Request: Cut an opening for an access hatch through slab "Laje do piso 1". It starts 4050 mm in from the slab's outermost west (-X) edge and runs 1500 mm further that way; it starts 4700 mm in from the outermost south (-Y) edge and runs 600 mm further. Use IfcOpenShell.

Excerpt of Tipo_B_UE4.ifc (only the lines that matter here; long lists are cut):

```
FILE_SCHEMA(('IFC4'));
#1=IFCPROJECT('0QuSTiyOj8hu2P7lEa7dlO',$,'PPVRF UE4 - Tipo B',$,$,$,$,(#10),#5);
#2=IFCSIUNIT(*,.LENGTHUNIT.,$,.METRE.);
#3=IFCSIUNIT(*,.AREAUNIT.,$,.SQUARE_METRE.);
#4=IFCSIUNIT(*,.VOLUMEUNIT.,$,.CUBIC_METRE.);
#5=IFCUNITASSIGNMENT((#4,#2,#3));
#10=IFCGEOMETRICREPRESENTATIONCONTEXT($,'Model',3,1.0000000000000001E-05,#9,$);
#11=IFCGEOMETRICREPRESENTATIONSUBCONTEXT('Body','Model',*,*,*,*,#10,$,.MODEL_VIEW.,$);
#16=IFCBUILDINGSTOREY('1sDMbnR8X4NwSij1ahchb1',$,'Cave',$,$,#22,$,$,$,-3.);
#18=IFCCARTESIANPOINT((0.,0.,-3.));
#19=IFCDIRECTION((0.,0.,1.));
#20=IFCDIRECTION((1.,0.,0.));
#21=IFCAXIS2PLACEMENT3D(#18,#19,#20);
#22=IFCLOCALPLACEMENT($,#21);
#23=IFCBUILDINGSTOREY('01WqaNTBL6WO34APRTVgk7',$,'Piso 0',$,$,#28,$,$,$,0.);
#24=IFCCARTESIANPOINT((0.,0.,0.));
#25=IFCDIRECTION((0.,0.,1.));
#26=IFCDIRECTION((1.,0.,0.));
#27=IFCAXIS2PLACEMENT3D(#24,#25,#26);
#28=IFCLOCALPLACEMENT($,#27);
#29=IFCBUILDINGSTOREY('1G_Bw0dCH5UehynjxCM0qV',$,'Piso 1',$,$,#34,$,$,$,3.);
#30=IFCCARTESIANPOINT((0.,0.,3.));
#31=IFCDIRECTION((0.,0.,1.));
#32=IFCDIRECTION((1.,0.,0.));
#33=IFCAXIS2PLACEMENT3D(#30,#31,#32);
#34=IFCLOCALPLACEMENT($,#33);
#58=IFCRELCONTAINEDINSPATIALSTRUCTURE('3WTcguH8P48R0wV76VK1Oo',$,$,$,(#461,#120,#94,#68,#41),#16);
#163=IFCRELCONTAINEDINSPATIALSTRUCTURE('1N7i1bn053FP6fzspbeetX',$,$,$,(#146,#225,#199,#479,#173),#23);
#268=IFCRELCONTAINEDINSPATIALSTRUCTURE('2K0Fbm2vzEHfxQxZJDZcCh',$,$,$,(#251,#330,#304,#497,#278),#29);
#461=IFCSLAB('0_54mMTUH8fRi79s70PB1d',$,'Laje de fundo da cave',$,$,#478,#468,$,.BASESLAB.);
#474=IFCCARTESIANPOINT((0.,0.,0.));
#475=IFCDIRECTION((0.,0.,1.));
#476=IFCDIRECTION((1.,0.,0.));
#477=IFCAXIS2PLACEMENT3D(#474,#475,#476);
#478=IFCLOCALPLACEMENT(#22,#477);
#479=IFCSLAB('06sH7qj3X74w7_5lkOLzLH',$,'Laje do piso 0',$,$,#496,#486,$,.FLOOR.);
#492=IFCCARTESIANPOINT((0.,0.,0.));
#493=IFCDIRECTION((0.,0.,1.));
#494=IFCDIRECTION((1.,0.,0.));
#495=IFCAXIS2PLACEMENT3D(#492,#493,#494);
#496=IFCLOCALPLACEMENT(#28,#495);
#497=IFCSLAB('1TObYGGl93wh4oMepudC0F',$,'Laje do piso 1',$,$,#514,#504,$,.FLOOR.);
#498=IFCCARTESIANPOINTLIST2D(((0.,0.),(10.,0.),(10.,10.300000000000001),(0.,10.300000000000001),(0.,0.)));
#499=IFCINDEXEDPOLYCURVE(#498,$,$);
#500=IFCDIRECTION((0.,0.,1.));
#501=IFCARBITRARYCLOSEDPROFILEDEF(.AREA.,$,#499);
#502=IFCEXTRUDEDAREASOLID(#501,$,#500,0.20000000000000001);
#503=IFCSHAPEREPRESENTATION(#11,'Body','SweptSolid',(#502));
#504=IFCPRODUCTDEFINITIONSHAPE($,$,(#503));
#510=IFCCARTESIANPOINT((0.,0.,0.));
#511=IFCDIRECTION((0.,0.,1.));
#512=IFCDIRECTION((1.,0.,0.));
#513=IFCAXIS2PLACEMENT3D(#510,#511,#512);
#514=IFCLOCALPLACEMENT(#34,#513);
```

```python
import numpy as np
import ifcopenshell
import ifcopenshell.api.feature
import ifcopenshell.api.geometry
import ifcopenshell.api.root
import ifcopenshell.geom
import ifcopenshell.util.placement
import ifcopenshell.util.representation
import ifcopenshell.util.shape
import ifcopenshell.util.unit

model = ifcopenshell.open("Tipo_B_UE4.ifc")
unit_scale = ifcopenshell.util.unit.calculate_unit_scale(model)
settings = ifcopenshell.geom.settings()


def volume(element):
    """Net volume in cubic metres, openings subtracted."""
    shape = ifcopenshell.geom.create_shape(settings, element)
    return ifcopenshell.util.shape.get_volume(shape.geometry)


slab = model.by_guid("1TObYGGl93wh4oMepudC0F")
before = volume(slab)

# Extent in the slab's own axes, in metres. The edges named are its -X and -Y sides.
slab_shape = ifcopenshell.geom.create_shape(settings, slab)
vertices = ifcopenshell.util.shape.get_vertices(slab_shape.geometry)
x_min, y_min, bottom = vertices.min(axis=0)
top = vertices[:, 2].max()

opening = ifcopenshell.api.root.create_entity(model, ifc_class="IfcOpeningElement", name="Access hatch opening", predefined_type="OPENING")
context = ifcopenshell.util.representation.get_context(model, "Model", "Body", "MODEL_VIEW")
width, depth = 1.5, 0.6
outline = [(0.0, 0.0), (width, 0.0), (width, depth), (0.0, depth), (0.0, 0.0)]
# Overshoot both faces by 50 mm so the cut is clean.
shape = ifcopenshell.api.geometry.add_slab_representation(
    model, context=context, depth=top - bottom + 0.1, polyline=outline
)
ifcopenshell.api.geometry.assign_representation(model, product=opening, representation=shape)

matrix = ifcopenshell.util.placement.get_local_placement(slab.ObjectPlacement)
matrix[:, 3] = matrix @ np.append(np.array([x_min + 4.05, y_min + 4.7, bottom - 0.05]) / unit_scale, 1.0)
ifcopenshell.api.geometry.edit_object_placement(model, product=opening, matrix=matrix, is_si=False)
ifcopenshell.api.feature.add_feature(model, feature=opening, element=slab)

after = volume(slab)

print(f"slab volume {before:.3f} -> {after:.3f} m3")

model.write("Tipo_B_UE4_edited.ifc")
```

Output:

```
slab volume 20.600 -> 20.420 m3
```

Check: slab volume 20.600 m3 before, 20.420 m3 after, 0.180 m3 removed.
